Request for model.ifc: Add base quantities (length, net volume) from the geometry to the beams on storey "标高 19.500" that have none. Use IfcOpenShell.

First a look at what the model holds.

```python
import ifcopenshell
import ifcopenshell.util.element
import ifcopenshell.util.unit

model = ifcopenshell.open("model.ifc")
print(model.schema)
for unit_type in ("LENGTHUNIT", "AREAUNIT", "VOLUMEUNIT"):
    print(unit_type, ifcopenshell.util.unit.calculate_unit_scale(model, unit_type))
storey = next(s for s in model.by_type("IfcBuildingStorey") if s.Name == "标高 19.500")
beams = [e for e in ifcopenshell.util.element.get_decomposition(storey) if e.is_a("IfcBeam")]
for e in sorted(beams, key=lambda e: e.id()):
    print(e.id(), e.is_a(), e.Name, list(ifcopenshell.util.element.get_psets(e, qtos_only=True)), sep=" | ")
```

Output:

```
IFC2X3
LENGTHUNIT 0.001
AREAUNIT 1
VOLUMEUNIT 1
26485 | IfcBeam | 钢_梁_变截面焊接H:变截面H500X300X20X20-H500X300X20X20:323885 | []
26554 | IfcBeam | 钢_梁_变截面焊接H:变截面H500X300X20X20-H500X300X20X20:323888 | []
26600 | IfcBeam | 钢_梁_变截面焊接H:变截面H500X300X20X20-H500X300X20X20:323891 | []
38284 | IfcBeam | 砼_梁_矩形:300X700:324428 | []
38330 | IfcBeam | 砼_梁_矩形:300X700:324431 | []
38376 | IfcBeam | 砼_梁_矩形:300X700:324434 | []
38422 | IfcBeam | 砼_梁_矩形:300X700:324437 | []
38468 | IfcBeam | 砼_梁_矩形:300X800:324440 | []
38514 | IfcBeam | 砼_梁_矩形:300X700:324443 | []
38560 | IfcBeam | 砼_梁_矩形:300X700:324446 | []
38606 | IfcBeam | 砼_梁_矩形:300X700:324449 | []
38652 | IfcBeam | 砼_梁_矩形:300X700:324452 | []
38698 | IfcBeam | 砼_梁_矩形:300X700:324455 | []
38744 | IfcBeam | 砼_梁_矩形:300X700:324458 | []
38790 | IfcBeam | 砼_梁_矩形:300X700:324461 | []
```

```python
import ifcopenshell
import ifcopenshell.api.pset
import ifcopenshell.geom
import ifcopenshell.util.element
import ifcopenshell.util.shape
import ifcopenshell.util.unit

model = ifcopenshell.open("model.ifc")
unit_scale = ifcopenshell.util.unit.calculate_unit_scale(model)
volume_scale = ifcopenshell.util.unit.calculate_unit_scale(model, "VOLUMEUNIT")
settings = ifcopenshell.geom.settings()

storey = next(s for s in model.by_type("IfcBuildingStorey") if s.Name == "标高 19.500")
beams = [e for e in ifcopenshell.util.element.get_decomposition(storey) if e.is_a("IfcBeam")]

for e in sorted(beams, key=lambda e: e.id()):
    if ifcopenshell.util.element.get_psets(e, qtos_only=True, should_inherit=False):
        continue
    # Geometry comes back in metres, in the element's own axes.
    shape = ifcopenshell.geom.create_shape(settings, e)
    values = {
        "Length": ifcopenshell.util.shape.get_max_xyz(shape.geometry) / unit_scale,
        "NetVolume": ifcopenshell.util.shape.get_volume(shape.geometry) / volume_scale,
    }
    qto = ifcopenshell.api.pset.add_qto(model, product=e, name="BaseQuantities")
    ifcopenshell.api.pset.edit_qto(model, qto=qto, properties=values)
    print(e.id(), {k: round(v, 3) for k, v in values.items()})

model.write("model_updated.ifc")
```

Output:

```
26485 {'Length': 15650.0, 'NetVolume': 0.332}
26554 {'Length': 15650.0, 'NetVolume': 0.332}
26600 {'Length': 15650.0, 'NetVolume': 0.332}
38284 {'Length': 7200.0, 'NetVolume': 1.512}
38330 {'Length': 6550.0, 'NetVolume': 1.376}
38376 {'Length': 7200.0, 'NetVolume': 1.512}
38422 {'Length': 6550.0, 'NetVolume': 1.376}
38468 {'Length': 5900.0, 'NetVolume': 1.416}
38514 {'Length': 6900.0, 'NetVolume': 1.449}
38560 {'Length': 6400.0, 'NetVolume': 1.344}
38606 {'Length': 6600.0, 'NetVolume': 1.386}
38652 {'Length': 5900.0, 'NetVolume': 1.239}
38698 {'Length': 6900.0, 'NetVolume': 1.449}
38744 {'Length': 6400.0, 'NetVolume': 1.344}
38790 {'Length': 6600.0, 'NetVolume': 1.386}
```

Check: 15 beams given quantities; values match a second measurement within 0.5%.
